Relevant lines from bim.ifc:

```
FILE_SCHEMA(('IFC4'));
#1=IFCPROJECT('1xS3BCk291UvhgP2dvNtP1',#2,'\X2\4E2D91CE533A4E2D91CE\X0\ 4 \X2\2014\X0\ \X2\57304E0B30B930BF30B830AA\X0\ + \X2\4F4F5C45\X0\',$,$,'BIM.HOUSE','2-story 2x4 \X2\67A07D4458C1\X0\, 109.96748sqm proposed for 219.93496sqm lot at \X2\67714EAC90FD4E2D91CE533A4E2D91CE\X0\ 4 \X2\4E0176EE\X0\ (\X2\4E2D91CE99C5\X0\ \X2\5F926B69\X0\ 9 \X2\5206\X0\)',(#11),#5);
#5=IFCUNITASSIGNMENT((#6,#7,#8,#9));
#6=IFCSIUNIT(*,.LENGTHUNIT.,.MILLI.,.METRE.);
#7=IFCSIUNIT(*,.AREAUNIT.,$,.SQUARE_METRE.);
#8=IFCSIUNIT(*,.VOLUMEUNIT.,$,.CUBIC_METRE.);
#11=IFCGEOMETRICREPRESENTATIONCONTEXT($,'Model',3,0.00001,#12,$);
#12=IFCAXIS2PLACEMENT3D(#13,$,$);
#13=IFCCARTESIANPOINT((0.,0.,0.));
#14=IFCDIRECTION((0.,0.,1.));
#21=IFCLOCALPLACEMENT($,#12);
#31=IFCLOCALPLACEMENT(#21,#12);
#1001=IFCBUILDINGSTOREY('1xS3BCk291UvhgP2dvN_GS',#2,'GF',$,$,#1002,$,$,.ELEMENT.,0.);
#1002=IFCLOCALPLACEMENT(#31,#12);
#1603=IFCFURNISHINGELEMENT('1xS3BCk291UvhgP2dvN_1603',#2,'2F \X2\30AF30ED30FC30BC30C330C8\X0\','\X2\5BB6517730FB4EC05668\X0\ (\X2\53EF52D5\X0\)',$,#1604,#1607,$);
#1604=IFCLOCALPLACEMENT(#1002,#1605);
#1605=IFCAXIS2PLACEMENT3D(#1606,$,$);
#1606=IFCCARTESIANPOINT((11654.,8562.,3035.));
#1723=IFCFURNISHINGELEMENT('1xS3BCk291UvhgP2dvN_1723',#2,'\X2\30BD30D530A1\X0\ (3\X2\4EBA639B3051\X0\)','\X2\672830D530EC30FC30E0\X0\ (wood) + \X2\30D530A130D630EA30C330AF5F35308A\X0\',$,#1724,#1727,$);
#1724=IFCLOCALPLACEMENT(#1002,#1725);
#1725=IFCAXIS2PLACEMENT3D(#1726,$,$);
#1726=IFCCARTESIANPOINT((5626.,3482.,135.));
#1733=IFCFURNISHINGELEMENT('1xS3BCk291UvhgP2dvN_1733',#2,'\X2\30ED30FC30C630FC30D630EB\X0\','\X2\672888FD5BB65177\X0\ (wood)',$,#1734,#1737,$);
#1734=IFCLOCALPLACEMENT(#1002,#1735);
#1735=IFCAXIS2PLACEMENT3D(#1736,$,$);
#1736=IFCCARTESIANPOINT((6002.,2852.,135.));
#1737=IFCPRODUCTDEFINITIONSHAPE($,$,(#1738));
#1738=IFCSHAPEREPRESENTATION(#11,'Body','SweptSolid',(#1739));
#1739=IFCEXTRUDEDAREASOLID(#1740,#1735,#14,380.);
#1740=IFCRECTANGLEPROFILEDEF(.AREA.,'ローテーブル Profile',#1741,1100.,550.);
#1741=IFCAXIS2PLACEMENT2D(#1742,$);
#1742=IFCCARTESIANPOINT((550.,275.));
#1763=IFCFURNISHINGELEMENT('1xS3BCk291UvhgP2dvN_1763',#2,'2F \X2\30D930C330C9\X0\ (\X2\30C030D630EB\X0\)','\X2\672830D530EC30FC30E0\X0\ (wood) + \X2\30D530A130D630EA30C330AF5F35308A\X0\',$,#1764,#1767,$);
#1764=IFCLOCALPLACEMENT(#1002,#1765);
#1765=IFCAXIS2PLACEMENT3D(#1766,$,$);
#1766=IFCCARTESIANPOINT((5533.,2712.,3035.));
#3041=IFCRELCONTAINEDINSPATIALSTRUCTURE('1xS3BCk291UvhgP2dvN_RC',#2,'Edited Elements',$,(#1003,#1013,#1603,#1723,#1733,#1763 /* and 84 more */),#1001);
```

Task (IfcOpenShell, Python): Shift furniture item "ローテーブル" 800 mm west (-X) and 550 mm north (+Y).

```python
import ifcopenshell
import ifcopenshell.api.geometry
import ifcopenshell.util.placement
import ifcopenshell.util.unit

model = ifcopenshell.open("bim.ifc")
unit_scale = ifcopenshell.util.unit.calculate_unit_scale(model)

item = model.by_guid("1xS3BCk291UvhgP2dvN_1733")
matrix = ifcopenshell.util.placement.get_local_placement(item.ObjectPlacement)
matrix[0, 3] -= 0.8 / unit_scale
matrix[1, 3] += 0.55 / unit_scale
ifcopenshell.api.geometry.edit_object_placement(model, product=item, matrix=matrix, is_si=False)

print(ifcopenshell.util.placement.get_local_placement(item.ObjectPlacement).round(3) + 0.0)

model.write("bim_v2.ifc")
```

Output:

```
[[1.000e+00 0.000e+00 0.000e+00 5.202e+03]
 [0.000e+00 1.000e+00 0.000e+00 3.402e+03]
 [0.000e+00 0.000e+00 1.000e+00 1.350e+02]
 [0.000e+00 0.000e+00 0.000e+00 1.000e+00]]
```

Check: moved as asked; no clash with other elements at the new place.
